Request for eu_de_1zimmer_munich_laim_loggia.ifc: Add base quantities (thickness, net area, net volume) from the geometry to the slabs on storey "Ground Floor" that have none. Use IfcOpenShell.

First a look at what the model holds.

```python
import ifcopenshell
import ifcopenshell.util.element
import ifcopenshell.util.unit

model = ifcopenshell.open("eu_de_1zimmer_munich_laim_loggia.ifc")
print(model.schema)
for unit_type in ("LENGTHUNIT", "AREAUNIT", "VOLUMEUNIT"):
    print(unit_type, ifcopenshell.util.unit.calculate_unit_scale(model, unit_type))
storey = next(s for s in model.by_type("IfcBuildingStorey") if s.Name == "Ground Floor")
slabs = [e for e in ifcopenshell.util.element.get_decomposition(storey) if e.is_a("IfcSlab")]
for e in sorted(slabs, key=lambda e: e.id()):
    print(e.id(), e.is_a(), e.Name, list(ifcopenshell.util.element.get_psets(e, qtos_only=True)), sep=" | ")
```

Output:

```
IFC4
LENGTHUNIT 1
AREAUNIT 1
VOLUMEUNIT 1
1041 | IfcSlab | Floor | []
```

```python
import ifcopenshell
import ifcopenshell.api.pset
import ifcopenshell.geom
import ifcopenshell.util.element
import ifcopenshell.util.shape
import ifcopenshell.util.unit

model = ifcopenshell.open("eu_de_1zimmer_munich_laim_loggia.ifc")
unit_scale = ifcopenshell.util.unit.calculate_unit_scale(model)
area_scale = ifcopenshell.util.unit.calculate_unit_scale(model, "AREAUNIT")
volume_scale = ifcopenshell.util.unit.calculate_unit_scale(model, "VOLUMEUNIT")
settings = ifcopenshell.geom.settings()

storey = next(s for s in model.by_type("IfcBuildingStorey") if s.Name == "Ground Floor")
slabs = [e for e in ifcopenshell.util.element.get_decomposition(storey) if e.is_a("IfcSlab")]

for e in sorted(slabs, key=lambda e: e.id()):
    if ifcopenshell.util.element.get_psets(e, qtos_only=True, should_inherit=False):
        continue
    # Geometry comes back in metres, in the element's own axes.
    shape = ifcopenshell.geom.create_shape(settings, e)
    values = {
        "Width": ifcopenshell.util.shape.get_z(shape.geometry) / unit_scale,
        "NetArea": ifcopenshell.util.shape.get_footprint_area(shape.geometry) / area_scale,
        "NetVolume": ifcopenshell.util.shape.get_volume(shape.geometry) / volume_scale,
    }
    qto = ifcopenshell.api.pset.add_qto(model, product=e, name="Qto_SlabBaseQuantities")
    ifcopenshell.api.pset.edit_qto(model, qto=qto, properties=values)
    print(e.id(), {k: round(v, 3) for k, v in values.items()})

model.write("eu_de_1zimmer_munich_laim_loggia_v2.ifc")
```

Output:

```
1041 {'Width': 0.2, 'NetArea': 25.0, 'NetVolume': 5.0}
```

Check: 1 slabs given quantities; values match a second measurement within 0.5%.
